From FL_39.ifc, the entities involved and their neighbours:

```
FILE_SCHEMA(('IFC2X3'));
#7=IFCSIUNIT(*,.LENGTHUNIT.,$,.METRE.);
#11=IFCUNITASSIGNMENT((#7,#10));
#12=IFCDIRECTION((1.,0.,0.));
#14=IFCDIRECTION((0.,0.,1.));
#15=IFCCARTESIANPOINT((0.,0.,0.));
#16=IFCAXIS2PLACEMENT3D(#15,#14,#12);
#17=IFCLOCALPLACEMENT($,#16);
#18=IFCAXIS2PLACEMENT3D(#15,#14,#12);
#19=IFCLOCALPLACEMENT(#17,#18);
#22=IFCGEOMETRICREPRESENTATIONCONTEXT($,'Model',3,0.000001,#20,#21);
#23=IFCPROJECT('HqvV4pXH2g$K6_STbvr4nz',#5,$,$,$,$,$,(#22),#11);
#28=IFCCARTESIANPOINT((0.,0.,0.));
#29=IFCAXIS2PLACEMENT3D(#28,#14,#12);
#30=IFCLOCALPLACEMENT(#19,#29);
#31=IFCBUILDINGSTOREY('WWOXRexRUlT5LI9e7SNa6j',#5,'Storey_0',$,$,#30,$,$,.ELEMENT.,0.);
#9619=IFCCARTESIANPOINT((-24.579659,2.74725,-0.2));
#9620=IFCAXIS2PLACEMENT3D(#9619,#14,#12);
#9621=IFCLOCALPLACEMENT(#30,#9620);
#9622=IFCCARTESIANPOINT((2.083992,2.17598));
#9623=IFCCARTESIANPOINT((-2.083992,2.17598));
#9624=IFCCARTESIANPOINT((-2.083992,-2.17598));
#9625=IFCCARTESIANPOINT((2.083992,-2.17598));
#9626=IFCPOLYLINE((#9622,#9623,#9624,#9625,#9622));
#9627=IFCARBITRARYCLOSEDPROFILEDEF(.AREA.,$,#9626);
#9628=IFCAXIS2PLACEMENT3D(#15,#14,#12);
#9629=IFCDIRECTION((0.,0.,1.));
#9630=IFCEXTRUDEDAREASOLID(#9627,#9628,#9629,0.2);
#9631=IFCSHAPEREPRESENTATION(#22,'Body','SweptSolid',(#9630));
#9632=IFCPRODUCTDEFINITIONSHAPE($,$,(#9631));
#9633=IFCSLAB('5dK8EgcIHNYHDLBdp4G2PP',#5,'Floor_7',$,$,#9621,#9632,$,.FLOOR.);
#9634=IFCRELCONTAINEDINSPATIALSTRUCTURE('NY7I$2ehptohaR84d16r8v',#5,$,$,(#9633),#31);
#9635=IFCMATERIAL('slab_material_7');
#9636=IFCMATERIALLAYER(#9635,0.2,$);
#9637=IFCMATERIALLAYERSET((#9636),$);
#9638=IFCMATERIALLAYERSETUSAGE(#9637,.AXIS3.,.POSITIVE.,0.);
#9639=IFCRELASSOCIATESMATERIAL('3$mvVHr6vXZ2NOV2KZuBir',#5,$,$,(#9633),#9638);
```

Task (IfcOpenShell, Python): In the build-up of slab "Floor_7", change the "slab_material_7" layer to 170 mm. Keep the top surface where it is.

```python
import ifcopenshell
import ifcopenshell.util.element

model = ifcopenshell.open("FL_39.ifc")

layer_set = model.by_id(9637)
layer = next(l for l in layer_set.MaterialLayers if l.Material and l.Material.Name == "slab_material_7")
change = 0.17 - layer.LayerThickness
layer.LayerThickness += change

# Geometry does not follow the layer set by itself.
slabs = [e for e in ifcopenshell.util.element.get_elements_by_material(model, layer_set) if e.is_a("IfcSlab")]
for slab in sorted(slabs, key=lambda e: e.id()):
    body = next(r for r in slab.Representation.Representations if r.RepresentationIdentifier == "Body")
    solid = body.Items[0]
    old_depth = solid.Depth
    solid.Depth += change
    # Extruded upwards: lower the start of the extrusion so the top stays.
    x, y, z = solid.Position.Location.Coordinates
    solid.Position.Location = model.createIfcCartesianPoint((x, y, z - change))
    print(slab.id(), f"{old_depth:g} -> {solid.Depth:g}")

# The layers are counted up from the underside, which has moved.
for usage in {ifcopenshell.util.element.get_material(slab) for slab in slabs}:
    usage.OffsetFromReferenceLine -= change

model.write("FL_39_updated.ifc")
```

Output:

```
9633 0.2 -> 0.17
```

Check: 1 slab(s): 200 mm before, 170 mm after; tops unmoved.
